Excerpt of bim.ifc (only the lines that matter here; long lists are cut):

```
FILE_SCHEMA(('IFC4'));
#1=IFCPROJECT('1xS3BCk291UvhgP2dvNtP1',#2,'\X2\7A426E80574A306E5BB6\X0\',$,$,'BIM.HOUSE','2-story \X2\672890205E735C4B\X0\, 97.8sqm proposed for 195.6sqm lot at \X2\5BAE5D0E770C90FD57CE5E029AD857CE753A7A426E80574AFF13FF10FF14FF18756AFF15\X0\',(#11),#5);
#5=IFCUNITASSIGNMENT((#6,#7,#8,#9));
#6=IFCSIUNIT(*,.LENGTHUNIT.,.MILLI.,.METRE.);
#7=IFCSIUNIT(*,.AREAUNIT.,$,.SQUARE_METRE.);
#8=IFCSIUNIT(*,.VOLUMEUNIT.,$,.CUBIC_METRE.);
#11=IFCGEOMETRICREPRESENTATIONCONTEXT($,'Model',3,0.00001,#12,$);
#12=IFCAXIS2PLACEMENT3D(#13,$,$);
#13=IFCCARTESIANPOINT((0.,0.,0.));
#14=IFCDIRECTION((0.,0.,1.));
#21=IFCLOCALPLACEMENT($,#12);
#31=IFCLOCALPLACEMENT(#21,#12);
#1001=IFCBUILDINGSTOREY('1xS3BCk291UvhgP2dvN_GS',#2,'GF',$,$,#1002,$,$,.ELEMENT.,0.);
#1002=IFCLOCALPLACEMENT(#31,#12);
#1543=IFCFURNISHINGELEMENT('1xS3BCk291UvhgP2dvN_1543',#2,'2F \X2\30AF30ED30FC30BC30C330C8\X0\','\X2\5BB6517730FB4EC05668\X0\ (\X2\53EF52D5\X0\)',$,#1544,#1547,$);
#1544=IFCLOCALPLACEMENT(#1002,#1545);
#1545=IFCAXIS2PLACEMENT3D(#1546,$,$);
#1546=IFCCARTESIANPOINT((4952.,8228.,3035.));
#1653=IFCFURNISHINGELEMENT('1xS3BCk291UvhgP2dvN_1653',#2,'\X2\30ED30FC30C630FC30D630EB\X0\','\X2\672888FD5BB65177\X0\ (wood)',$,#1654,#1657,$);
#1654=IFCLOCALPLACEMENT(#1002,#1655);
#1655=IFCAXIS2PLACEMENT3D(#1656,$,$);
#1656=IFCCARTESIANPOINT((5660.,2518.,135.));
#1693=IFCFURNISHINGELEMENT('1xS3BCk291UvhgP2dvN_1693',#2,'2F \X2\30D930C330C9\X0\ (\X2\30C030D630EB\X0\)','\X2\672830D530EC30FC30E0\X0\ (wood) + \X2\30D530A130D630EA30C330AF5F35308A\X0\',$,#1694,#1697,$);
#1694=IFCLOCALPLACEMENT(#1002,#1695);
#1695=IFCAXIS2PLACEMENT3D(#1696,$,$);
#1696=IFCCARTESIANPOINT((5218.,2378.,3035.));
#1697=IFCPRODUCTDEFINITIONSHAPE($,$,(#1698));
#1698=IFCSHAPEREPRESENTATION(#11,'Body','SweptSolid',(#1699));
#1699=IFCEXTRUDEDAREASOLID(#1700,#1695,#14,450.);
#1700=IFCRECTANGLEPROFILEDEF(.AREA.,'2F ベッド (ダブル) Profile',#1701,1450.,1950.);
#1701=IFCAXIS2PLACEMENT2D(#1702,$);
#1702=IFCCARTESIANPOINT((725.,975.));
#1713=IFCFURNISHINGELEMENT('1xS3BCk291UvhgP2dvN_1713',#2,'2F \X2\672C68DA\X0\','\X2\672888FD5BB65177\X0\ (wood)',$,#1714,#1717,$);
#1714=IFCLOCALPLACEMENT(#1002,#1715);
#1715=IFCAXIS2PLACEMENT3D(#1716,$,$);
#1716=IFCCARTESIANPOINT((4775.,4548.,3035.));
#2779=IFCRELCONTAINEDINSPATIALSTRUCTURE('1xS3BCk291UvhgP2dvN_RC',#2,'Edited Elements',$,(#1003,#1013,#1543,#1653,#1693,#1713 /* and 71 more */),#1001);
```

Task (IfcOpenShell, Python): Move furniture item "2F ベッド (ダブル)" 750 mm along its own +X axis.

```python
import ifcopenshell
import ifcopenshell.api.geometry
import ifcopenshell.util.placement
import ifcopenshell.util.unit

model = ifcopenshell.open("bim.ifc")
unit_scale = ifcopenshell.util.unit.calculate_unit_scale(model)

item = model.by_guid("1xS3BCk291UvhgP2dvN_1693")
matrix = ifcopenshell.util.placement.get_local_placement(item.ObjectPlacement)
matrix[:3, 3] += matrix[:3, 0] * 0.75 / unit_scale
ifcopenshell.api.geometry.edit_object_placement(model, product=item, matrix=matrix, is_si=False)

print(ifcopenshell.util.placement.get_local_placement(item.ObjectPlacement).round(3) + 0.0)

model.write("bim_v2.ifc")
```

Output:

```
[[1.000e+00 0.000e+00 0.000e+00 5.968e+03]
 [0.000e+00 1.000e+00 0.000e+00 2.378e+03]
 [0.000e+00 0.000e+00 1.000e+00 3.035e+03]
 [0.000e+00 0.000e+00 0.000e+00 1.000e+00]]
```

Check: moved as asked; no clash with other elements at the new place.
